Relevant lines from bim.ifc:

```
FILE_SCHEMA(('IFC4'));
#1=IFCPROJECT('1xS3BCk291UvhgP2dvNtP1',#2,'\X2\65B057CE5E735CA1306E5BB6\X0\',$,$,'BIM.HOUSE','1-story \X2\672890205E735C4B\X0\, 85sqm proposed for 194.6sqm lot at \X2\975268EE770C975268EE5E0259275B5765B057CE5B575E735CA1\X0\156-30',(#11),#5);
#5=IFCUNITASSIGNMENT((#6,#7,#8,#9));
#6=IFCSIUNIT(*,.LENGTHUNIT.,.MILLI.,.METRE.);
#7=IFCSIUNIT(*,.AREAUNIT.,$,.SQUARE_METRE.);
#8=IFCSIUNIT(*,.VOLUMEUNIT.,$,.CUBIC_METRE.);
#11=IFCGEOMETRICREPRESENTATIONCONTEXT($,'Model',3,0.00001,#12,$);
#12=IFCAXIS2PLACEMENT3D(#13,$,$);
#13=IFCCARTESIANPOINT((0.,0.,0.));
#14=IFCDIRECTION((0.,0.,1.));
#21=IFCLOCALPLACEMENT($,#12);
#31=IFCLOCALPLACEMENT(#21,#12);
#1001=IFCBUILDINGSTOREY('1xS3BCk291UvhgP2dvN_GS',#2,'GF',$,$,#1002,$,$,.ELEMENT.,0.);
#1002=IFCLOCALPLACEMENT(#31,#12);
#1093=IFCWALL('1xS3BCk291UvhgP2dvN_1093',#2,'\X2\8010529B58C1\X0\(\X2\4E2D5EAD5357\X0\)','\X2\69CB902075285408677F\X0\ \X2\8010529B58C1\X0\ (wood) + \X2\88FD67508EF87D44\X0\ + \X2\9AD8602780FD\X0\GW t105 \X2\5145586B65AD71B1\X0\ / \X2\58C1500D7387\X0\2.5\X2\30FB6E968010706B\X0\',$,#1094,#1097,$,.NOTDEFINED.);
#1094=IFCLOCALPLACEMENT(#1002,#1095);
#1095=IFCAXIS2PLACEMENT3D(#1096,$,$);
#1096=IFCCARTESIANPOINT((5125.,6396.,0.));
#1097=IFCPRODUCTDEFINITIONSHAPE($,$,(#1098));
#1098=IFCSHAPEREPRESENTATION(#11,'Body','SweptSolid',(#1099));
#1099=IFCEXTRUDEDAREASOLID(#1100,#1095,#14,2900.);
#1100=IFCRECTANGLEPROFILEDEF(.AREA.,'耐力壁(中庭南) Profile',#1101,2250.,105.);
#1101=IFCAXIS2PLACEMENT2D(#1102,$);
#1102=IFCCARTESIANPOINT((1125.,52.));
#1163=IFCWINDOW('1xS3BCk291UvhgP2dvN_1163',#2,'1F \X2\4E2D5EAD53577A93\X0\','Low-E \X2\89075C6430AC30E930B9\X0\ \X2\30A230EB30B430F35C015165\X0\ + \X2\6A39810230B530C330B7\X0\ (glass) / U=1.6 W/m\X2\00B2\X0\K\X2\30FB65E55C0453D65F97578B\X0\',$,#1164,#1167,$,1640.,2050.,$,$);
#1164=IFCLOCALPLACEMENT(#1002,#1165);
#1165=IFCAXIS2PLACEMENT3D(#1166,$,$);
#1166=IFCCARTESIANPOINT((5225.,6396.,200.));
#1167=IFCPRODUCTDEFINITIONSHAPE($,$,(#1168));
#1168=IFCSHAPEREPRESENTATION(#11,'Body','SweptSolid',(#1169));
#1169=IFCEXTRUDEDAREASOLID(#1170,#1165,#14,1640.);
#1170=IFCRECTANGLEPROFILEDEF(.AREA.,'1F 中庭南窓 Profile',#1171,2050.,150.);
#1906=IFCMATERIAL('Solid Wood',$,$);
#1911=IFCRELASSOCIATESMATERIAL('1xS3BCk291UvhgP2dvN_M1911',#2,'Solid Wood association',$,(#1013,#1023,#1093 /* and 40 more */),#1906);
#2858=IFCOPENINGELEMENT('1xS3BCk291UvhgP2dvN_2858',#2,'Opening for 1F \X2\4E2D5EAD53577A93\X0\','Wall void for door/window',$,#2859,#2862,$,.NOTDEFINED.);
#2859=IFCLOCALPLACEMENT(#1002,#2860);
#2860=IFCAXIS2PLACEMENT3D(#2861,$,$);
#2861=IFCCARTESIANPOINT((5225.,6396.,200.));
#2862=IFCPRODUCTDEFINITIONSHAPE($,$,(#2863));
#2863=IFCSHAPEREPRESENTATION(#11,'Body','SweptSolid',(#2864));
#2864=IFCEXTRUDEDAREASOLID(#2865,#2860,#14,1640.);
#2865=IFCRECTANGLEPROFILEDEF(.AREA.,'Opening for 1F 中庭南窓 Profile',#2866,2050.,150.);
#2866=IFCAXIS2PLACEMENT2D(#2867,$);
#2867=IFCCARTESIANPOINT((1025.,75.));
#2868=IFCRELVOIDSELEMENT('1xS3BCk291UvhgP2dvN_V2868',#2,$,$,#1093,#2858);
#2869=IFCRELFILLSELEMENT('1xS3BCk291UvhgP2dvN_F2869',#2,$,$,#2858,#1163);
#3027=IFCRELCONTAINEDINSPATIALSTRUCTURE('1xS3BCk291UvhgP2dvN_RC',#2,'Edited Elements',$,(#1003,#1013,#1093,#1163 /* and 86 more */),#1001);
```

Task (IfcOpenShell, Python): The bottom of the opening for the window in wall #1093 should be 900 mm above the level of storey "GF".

```python
import numpy as np
import ifcopenshell
import ifcopenshell.api.geometry
import ifcopenshell.geom
import ifcopenshell.util.element
import ifcopenshell.util.placement
import ifcopenshell.util.shape
import ifcopenshell.util.unit

model = ifcopenshell.open("bim.ifc")
unit_scale = ifcopenshell.util.unit.calculate_unit_scale(model)

window = model.by_guid("1xS3BCk291UvhgP2dvN_1163")
opening = window.FillsVoids[0].RelatingOpeningElement
storey = ifcopenshell.util.element.get_container(window, ifc_class="IfcBuildingStorey")
level = ifcopenshell.util.placement.get_local_placement(storey.ObjectPlacement)[2, 3]

# The opening's origin need not be at the sill, so measure its lowest point.
shape = ifcopenshell.geom.create_shape(ifcopenshell.geom.settings(), opening)
bottom = ifcopenshell.util.shape.get_shape_bottom_elevation(shape, shape.geometry) / unit_scale
dz = level + 0.9 / unit_scale - bottom

shift = np.array([0.0, 0.0, dz])
# The window is not placed relative to its opening, so move both.
for product in (opening, window):
    matrix = ifcopenshell.util.placement.get_local_placement(product.ObjectPlacement)
    matrix[:3, 3] += shift
    ifcopenshell.api.geometry.edit_object_placement(model, product=product, matrix=matrix, is_si=False)

print(f"moved by {dz * unit_scale:+.3f} m")

model.write("bim-out.ifc")
```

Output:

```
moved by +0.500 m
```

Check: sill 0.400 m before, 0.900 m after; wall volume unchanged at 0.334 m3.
